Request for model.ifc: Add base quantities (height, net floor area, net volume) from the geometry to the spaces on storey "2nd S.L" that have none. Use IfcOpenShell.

First a look at what the model holds.

```python
import ifcopenshell
import ifcopenshell.util.element
import ifcopenshell.util.unit

model = ifcopenshell.open("model.ifc")
print(model.schema)
for unit_type in ("LENGTHUNIT", "AREAUNIT", "VOLUMEUNIT"):
    print(unit_type, ifcopenshell.util.unit.calculate_unit_scale(model, unit_type))
storey = next(s for s in model.by_type("IfcBuildingStorey") if s.Name == "2nd S.L")
spaces = [e for e in ifcopenshell.util.element.get_decomposition(storey) if e.is_a("IfcSpace")]
for e in sorted(spaces, key=lambda e: e.id()):
    print(e.id(), e.is_a(), e.Name, list(ifcopenshell.util.element.get_psets(e, qtos_only=True)), sep=" | ")
```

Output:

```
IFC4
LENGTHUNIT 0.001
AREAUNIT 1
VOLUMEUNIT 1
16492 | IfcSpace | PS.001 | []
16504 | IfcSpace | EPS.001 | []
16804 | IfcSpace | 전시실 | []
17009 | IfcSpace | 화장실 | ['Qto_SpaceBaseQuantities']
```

```python
import ifcopenshell
import ifcopenshell.api.pset
import ifcopenshell.geom
import ifcopenshell.util.element
import ifcopenshell.util.shape
import ifcopenshell.util.unit

model = ifcopenshell.open("model.ifc")
unit_scale = ifcopenshell.util.unit.calculate_unit_scale(model)
area_scale = ifcopenshell.util.unit.calculate_unit_scale(model, "AREAUNIT")
volume_scale = ifcopenshell.util.unit.calculate_unit_scale(model, "VOLUMEUNIT")
settings = ifcopenshell.geom.settings()

storey = next(s for s in model.by_type("IfcBuildingStorey") if s.Name == "2nd S.L")
spaces = [e for e in ifcopenshell.util.element.get_decomposition(storey) if e.is_a("IfcSpace")]

for e in sorted(spaces, key=lambda e: e.id()):
    if ifcopenshell.util.element.get_psets(e, qtos_only=True, should_inherit=False):
        continue
    # Geometry comes back in metres, in the element's own axes.
    shape = ifcopenshell.geom.create_shape(settings, e)
    values = {
        "Height": ifcopenshell.util.shape.get_z(shape.geometry) / unit_scale,
        "NetFloorArea": ifcopenshell.util.shape.get_footprint_area(shape.geometry) / area_scale,
        "NetVolume": ifcopenshell.util.shape.get_volume(shape.geometry) / volume_scale,
    }
    qto = ifcopenshell.api.pset.add_qto(model, product=e, name="Qto_SpaceBaseQuantities")
    ifcopenshell.api.pset.edit_qto(model, qto=qto, properties=values)
    print(e.id(), {k: round(v, 3) for k, v in values.items()})

model.write("model_v2.ifc")
```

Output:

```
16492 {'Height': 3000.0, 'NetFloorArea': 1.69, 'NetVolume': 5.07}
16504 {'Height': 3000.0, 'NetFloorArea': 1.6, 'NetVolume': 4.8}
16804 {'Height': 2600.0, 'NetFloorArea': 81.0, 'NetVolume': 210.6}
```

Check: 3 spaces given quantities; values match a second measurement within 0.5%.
